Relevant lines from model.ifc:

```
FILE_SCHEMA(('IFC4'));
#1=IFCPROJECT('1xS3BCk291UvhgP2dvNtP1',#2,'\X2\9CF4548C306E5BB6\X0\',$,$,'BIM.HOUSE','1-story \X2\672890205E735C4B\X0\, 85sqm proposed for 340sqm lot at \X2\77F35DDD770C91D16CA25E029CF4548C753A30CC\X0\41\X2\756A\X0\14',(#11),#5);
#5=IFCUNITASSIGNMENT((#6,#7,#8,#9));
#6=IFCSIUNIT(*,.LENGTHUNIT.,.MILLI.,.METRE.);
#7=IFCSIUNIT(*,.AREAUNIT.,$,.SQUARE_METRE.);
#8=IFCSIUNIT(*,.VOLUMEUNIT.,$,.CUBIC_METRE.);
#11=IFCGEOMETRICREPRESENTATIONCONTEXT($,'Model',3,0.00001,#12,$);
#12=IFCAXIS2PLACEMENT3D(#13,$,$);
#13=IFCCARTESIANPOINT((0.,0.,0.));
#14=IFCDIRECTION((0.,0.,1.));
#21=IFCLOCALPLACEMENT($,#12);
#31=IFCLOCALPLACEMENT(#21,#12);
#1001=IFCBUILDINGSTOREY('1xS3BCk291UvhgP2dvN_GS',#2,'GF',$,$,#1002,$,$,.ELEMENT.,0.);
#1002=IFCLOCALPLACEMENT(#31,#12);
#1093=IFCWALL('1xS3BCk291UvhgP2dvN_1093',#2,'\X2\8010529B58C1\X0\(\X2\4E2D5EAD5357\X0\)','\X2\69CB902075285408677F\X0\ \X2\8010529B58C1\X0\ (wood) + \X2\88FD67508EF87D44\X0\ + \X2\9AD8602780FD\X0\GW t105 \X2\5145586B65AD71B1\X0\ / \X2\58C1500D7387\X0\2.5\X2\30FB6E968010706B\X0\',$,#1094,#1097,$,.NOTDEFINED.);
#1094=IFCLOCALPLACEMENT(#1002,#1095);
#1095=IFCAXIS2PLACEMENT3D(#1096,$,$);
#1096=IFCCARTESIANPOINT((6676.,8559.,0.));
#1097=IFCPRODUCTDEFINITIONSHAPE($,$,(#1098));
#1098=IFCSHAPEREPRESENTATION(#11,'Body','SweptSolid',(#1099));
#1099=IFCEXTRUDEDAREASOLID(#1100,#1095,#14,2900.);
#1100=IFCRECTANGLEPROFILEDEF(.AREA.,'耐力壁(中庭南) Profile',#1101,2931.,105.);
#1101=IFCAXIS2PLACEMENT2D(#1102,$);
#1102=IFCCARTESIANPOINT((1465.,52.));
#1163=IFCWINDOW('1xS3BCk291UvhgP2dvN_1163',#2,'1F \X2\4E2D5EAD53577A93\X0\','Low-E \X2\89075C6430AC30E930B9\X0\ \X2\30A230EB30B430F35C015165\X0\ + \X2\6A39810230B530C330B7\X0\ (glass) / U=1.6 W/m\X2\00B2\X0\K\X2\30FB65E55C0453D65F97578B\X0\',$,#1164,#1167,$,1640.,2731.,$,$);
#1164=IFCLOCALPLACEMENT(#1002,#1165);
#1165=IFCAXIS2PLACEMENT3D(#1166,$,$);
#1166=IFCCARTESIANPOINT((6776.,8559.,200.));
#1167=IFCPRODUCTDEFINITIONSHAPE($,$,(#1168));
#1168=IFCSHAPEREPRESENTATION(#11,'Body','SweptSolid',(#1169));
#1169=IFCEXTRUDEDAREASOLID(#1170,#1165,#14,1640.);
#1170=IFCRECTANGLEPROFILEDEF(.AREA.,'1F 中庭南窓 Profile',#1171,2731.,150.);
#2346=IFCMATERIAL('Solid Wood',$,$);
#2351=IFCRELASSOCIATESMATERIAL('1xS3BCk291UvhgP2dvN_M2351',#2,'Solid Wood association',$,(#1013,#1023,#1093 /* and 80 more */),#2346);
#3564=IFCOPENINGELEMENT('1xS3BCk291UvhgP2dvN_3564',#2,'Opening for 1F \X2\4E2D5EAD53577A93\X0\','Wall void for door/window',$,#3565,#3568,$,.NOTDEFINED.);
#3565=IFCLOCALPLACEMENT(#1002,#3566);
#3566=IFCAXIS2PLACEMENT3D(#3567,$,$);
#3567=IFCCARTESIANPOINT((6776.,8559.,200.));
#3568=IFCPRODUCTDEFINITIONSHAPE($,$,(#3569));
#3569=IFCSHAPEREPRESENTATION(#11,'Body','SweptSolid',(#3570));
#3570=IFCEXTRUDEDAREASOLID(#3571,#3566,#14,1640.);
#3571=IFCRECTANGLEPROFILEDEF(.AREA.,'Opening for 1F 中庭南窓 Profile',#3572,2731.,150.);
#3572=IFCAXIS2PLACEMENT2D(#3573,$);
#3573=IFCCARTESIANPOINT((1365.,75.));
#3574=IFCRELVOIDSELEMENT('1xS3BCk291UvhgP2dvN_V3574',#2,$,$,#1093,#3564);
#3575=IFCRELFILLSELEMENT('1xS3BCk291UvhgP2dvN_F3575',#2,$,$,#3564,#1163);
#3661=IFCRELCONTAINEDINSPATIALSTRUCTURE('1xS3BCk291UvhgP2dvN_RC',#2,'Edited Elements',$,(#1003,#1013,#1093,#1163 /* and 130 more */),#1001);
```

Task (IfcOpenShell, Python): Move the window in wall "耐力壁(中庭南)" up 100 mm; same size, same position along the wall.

```python
import numpy as np
import ifcopenshell
import ifcopenshell.api.geometry
import ifcopenshell.util.placement
import ifcopenshell.util.unit

model = ifcopenshell.open("model.ifc")
unit_scale = ifcopenshell.util.unit.calculate_unit_scale(model)

window = model.by_guid("1xS3BCk291UvhgP2dvN_1163")
opening = window.FillsVoids[0].RelatingOpeningElement
dz = 0.1 / unit_scale

shift = np.array([0.0, 0.0, dz])
# The window is not placed relative to its opening, so move both.
for product in (opening, window):
    matrix = ifcopenshell.util.placement.get_local_placement(product.ObjectPlacement)
    matrix[:3, 3] += shift
    ifcopenshell.api.geometry.edit_object_placement(model, product=product, matrix=matrix, is_si=False)

print(f"moved by {dz * unit_scale:+.3f} m")

model.write("model_rev.ifc")
```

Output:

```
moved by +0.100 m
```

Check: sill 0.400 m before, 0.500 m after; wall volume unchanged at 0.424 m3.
